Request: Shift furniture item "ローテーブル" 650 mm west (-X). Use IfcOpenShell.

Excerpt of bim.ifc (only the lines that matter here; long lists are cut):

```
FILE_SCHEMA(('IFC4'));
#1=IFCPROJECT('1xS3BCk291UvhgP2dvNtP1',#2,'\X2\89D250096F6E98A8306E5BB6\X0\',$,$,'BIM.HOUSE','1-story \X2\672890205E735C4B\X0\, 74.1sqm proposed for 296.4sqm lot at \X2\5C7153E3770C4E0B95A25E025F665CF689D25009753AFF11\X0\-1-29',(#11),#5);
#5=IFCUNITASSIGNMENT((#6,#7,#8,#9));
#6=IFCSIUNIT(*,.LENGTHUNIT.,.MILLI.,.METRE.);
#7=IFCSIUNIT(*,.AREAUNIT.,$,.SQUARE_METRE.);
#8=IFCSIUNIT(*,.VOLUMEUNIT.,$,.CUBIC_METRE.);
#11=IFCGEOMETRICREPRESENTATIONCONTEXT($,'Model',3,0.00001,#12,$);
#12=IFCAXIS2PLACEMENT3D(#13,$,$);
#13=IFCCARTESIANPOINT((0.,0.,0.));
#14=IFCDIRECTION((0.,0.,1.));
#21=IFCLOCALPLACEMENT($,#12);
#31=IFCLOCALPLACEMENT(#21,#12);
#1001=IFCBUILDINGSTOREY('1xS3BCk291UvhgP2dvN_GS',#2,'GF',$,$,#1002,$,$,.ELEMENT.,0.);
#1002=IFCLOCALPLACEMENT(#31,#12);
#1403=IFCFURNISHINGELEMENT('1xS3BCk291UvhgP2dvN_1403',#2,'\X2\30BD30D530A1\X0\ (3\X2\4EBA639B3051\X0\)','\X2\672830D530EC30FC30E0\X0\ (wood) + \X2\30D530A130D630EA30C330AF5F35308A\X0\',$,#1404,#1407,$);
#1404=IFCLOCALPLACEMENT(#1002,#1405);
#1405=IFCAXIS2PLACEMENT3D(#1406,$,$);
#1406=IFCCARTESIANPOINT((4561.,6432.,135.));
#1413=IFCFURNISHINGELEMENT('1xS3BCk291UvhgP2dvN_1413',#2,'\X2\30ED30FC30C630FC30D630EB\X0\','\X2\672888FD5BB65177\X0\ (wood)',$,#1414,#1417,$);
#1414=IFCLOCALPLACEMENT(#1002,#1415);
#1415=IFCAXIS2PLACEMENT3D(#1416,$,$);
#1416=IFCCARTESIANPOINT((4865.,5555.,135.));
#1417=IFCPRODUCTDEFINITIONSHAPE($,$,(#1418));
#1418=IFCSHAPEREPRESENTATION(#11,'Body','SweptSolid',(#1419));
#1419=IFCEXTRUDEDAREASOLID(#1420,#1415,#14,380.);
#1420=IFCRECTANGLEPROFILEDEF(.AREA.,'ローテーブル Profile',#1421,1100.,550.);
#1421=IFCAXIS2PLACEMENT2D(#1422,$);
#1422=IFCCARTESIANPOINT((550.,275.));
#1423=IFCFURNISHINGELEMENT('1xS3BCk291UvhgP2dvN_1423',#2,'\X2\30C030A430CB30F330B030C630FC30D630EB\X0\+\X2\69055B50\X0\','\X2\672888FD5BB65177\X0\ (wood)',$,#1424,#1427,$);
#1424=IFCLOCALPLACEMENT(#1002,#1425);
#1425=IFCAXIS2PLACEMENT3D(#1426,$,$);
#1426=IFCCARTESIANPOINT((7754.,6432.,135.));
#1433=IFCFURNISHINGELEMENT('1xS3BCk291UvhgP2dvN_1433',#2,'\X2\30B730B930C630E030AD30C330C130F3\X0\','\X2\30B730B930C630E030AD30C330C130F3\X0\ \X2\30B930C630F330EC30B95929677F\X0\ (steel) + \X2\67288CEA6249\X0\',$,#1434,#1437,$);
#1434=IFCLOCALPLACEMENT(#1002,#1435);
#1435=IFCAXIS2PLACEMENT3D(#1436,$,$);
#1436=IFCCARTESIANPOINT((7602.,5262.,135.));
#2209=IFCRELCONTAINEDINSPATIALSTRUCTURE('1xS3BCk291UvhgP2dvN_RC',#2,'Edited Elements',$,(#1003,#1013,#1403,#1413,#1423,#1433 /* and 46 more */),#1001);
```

```python
import ifcopenshell
import ifcopenshell.api.geometry
import ifcopenshell.util.placement

model = ifcopenshell.open("bim.ifc")

item = model.by_guid("1xS3BCk291UvhgP2dvN_1413")
matrix = ifcopenshell.util.placement.get_local_placement(item.ObjectPlacement)
matrix[0, 3] -= 650.0
ifcopenshell.api.geometry.edit_object_placement(model, product=item, matrix=matrix, is_si=False)

print(ifcopenshell.util.placement.get_local_placement(item.ObjectPlacement).round(3) + 0.0)

model.write("bim-out.ifc")
```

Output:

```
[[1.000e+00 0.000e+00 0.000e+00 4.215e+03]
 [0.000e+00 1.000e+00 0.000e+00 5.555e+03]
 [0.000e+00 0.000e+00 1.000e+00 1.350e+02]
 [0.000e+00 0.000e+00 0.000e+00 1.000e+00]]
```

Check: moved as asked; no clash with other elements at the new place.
